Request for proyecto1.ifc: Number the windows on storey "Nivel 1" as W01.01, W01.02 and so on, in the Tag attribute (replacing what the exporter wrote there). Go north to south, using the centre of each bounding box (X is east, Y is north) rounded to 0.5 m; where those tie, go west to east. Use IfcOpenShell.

First a look at what the model holds.

```python
import ifcopenshell
import ifcopenshell.util.element
import ifcopenshell.util.placement

model = ifcopenshell.open("proyecto1.ifc")
print(model.schema)
storey = next(s for s in model.by_type("IfcBuildingStorey") if s.Name == "Nivel 1")
windows = [e for e in ifcopenshell.util.element.get_decomposition(storey) if e.is_a("IfcWindow")]
for e in sorted(windows, key=lambda e: e.id()):
    origin = ifcopenshell.util.placement.get_local_placement(e.ObjectPlacement)[:3, 3]
    print(e.id(), e.Tag, e.Name, origin.round(2) + 0.0, sep=" | ")
```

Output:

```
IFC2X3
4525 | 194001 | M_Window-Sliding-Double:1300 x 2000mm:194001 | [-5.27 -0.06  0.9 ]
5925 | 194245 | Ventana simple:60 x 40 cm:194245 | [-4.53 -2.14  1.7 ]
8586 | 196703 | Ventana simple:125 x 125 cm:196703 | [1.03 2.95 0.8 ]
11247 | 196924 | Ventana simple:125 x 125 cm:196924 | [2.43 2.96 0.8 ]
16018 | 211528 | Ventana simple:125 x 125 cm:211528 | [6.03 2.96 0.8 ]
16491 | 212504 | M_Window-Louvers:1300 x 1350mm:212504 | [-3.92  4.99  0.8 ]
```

```python
import ifcopenshell
import ifcopenshell.geom
import ifcopenshell.util.element
import ifcopenshell.util.shape

model = ifcopenshell.open("proyecto1.ifc")
settings = ifcopenshell.geom.settings()
settings.set("use-world-coords", True)


def centre(element):
    shape = ifcopenshell.geom.create_shape(settings, element)
    return ifcopenshell.util.shape.get_bbox_centroid(shape.geometry)


storey = next(s for s in model.by_type("IfcBuildingStorey") if s.Name == "Nivel 1")
windows = [e for e in ifcopenshell.util.element.get_decomposition(storey) if e.is_a("IfcWindow")]

# Insertion points can sit at a corner or the storey origin, so sort by the geometry (in metres).
centres = {e: centre(e) for e in windows}
windows.sort(key=lambda e: (-round(centres[e][1] / 0.5), centres[e][0]))

for i, e in enumerate(windows, start=1):
    number = f"W01.{i:02d}"
    e.Tag = number
    print(e.id(), number)

model.write("proyecto1_rev.ifc")
```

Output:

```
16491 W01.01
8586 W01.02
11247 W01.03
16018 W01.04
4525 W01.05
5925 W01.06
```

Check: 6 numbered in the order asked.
